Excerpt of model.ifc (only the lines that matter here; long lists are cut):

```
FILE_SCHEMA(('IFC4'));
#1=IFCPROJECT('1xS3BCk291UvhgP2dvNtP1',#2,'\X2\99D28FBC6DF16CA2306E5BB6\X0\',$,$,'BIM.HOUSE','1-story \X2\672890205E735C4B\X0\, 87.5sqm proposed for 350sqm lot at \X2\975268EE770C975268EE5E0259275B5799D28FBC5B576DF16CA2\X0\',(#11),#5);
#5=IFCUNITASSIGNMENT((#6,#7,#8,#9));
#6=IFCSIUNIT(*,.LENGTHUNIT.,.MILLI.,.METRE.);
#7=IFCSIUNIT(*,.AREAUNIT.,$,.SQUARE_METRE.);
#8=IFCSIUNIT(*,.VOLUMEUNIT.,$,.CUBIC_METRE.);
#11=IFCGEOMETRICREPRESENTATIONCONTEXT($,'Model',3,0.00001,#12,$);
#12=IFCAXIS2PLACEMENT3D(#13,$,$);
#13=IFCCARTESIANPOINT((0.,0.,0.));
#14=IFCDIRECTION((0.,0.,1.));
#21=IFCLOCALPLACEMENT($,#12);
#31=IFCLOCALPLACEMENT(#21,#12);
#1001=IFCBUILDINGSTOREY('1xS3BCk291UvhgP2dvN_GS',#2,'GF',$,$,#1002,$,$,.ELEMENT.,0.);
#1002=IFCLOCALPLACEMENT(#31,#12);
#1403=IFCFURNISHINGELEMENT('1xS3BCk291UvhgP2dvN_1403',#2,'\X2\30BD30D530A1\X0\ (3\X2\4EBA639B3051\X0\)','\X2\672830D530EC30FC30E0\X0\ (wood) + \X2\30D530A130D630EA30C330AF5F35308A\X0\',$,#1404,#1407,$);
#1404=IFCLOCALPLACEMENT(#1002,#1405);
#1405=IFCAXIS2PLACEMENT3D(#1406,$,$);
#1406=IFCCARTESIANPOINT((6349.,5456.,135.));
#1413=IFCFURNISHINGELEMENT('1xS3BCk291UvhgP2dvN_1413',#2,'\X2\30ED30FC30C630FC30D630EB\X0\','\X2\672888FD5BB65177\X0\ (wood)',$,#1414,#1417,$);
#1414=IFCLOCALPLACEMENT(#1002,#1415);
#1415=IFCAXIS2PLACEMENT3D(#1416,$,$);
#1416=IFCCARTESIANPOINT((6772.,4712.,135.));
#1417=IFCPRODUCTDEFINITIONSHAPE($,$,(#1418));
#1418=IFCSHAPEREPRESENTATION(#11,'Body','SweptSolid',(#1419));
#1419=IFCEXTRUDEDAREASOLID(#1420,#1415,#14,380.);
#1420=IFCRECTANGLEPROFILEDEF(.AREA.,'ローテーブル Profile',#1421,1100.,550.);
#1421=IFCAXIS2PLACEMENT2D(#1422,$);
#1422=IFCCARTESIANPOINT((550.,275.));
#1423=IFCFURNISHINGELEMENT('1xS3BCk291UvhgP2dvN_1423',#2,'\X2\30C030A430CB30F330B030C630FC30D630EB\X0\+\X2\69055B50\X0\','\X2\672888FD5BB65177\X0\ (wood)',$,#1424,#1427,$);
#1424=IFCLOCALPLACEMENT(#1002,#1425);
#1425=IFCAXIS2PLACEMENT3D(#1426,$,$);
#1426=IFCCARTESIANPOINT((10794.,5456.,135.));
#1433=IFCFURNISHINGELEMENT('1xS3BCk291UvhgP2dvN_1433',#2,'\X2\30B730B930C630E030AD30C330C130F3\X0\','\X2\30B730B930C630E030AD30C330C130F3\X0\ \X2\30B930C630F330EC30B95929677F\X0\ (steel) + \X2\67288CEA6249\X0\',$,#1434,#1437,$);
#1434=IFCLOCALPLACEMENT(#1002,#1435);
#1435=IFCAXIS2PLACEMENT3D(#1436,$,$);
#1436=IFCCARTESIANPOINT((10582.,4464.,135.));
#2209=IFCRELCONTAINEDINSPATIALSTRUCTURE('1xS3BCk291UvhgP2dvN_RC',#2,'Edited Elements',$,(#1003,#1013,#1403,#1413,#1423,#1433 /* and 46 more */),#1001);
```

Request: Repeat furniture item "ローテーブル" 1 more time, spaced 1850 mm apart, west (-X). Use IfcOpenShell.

```python
import numpy as np
import ifcopenshell
import ifcopenshell.api.geometry
import ifcopenshell.api.root
import ifcopenshell.util.element
import ifcopenshell.util.placement

model = ifcopenshell.open("model.ifc")


def reuse_history(source, copy):
    """copy_class also copies each property set's owner history, people and application; keep the originals."""
    for rel in copy.IsDefinedBy:
        if rel.is_a("IfcRelDefinesByProperties") and (history := rel.RelatingPropertyDefinition.OwnerHistory):
            rel.RelatingPropertyDefinition.OwnerHistory = source.OwnerHistory
            ifcopenshell.util.element.remove_deep2(model, history)


source = model.by_id(1413)
base = ifcopenshell.util.placement.get_local_placement(source.ObjectPlacement)
step = np.array([-1.0, 0.0, 0.0]) * 1850.0

for i in range(1, 2):
    copy = ifcopenshell.api.root.copy_class(model, product=source)
    copy.Representation = ifcopenshell.util.element.copy_deep(
        model, source.Representation, exclude=["IfcGeometricRepresentationContext", "IfcRepresentationMap"]
    )
    reuse_history(source, copy)
    matrix = base.copy()
    matrix[:3, 3] += i * step
    print("added at", matrix[:3, 3].round(3) + 0.0)
    ifcopenshell.api.geometry.edit_object_placement(model, product=copy, matrix=matrix, is_si=False)

model.write("model_rev.ifc")
```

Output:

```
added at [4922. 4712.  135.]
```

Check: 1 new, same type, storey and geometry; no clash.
